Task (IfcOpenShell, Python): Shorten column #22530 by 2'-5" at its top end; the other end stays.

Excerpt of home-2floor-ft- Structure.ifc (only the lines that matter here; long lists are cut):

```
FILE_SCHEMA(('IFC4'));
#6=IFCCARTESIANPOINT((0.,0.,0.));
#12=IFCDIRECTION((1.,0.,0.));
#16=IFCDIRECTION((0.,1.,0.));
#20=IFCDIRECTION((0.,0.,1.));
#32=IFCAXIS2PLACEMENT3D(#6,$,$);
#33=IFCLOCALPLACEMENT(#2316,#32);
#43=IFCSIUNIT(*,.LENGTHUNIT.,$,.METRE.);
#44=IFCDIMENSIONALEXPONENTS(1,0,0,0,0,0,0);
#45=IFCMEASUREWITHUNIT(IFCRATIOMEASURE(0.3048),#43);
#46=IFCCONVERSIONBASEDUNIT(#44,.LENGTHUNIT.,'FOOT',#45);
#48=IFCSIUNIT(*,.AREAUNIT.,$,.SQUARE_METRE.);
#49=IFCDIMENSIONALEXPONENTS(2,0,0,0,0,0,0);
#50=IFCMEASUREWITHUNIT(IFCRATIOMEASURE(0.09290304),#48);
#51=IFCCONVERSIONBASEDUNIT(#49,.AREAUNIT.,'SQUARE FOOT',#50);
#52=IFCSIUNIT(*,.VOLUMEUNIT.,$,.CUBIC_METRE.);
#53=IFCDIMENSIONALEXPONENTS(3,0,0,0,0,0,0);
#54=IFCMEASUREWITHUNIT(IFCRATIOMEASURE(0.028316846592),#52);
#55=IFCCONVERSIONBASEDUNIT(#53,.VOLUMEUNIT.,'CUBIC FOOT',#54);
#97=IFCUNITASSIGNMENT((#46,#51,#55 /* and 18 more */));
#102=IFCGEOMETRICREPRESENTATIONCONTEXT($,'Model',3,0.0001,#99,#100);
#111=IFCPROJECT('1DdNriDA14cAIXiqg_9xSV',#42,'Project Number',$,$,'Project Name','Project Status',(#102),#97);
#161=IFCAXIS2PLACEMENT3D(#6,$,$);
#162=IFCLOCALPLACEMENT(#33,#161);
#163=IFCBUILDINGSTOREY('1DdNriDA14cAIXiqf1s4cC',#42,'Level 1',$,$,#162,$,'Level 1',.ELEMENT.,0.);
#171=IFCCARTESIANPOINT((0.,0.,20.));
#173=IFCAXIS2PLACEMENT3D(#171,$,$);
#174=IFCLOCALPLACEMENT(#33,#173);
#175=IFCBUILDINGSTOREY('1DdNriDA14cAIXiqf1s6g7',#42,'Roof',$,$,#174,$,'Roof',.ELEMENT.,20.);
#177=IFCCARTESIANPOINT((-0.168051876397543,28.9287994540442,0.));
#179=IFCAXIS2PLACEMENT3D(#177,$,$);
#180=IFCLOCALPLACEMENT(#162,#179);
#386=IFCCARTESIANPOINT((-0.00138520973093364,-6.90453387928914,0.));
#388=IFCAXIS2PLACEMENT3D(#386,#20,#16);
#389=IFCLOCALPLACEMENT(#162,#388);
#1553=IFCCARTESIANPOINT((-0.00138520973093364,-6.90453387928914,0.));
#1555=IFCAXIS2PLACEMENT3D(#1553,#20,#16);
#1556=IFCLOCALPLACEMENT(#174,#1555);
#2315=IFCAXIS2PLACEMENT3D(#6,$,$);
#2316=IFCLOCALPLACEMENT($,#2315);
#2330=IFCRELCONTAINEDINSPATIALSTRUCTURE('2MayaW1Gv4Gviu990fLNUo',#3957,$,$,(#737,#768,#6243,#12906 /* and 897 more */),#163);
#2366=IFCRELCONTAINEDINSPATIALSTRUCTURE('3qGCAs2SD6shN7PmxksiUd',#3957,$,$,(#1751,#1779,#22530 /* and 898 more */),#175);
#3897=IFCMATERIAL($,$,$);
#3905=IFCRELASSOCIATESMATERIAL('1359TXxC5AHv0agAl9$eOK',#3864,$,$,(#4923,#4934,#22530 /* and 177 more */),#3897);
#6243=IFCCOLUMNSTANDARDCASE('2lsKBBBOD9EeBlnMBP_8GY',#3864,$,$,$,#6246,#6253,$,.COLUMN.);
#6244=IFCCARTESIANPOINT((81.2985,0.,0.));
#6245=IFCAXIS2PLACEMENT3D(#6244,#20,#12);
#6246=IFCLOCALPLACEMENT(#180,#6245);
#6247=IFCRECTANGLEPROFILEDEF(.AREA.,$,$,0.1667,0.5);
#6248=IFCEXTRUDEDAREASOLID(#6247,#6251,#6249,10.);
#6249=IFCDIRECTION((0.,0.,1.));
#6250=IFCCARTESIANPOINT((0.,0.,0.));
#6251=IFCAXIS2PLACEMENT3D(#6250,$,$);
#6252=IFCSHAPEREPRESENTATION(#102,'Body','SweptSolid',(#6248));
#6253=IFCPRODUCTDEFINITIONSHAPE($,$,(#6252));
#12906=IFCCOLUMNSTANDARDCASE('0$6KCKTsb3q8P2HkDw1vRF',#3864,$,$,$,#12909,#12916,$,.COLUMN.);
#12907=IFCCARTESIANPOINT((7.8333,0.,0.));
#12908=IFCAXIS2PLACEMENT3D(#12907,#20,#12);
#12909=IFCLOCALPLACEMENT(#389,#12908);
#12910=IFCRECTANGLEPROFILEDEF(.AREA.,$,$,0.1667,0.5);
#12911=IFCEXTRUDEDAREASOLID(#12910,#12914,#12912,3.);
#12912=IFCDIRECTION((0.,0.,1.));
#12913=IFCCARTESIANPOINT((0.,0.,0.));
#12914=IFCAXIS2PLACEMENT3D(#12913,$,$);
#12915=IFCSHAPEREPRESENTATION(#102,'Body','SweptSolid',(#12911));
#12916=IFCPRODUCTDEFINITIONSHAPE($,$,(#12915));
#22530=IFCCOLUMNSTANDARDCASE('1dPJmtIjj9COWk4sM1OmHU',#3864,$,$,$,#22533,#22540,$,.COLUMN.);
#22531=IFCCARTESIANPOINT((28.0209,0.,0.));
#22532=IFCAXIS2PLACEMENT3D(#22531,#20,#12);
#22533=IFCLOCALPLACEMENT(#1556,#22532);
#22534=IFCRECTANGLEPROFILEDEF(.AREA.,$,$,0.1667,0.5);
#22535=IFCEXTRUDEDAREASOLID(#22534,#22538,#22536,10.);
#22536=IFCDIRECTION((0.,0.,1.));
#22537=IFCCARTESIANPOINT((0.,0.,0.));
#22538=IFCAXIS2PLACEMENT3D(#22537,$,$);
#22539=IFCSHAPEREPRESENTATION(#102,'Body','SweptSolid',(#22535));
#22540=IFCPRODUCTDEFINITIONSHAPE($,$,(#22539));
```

```python
import ifcopenshell
import ifcopenshell.util.unit

model = ifcopenshell.open("home-2floor-ft- Structure.ifc")
unit_scale = ifcopenshell.util.unit.calculate_unit_scale(model)

member = model.by_guid("1dPJmtIjj9COWk4sM1OmHU")
change = -29 * 0.0254 / unit_scale

# The extrusion runs towards the end named, so only its depth changes.
body = next(r for r in member.Representation.Representations if r.RepresentationIdentifier == "Body")
solid = body.Items[0]
old_length = solid.Depth
solid.Depth += change

print(f"length {old_length:g} -> {solid.Depth:g}")

model.write("home-2floor-ft- Structure-out.ifc")
```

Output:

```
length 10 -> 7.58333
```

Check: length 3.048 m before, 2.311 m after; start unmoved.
